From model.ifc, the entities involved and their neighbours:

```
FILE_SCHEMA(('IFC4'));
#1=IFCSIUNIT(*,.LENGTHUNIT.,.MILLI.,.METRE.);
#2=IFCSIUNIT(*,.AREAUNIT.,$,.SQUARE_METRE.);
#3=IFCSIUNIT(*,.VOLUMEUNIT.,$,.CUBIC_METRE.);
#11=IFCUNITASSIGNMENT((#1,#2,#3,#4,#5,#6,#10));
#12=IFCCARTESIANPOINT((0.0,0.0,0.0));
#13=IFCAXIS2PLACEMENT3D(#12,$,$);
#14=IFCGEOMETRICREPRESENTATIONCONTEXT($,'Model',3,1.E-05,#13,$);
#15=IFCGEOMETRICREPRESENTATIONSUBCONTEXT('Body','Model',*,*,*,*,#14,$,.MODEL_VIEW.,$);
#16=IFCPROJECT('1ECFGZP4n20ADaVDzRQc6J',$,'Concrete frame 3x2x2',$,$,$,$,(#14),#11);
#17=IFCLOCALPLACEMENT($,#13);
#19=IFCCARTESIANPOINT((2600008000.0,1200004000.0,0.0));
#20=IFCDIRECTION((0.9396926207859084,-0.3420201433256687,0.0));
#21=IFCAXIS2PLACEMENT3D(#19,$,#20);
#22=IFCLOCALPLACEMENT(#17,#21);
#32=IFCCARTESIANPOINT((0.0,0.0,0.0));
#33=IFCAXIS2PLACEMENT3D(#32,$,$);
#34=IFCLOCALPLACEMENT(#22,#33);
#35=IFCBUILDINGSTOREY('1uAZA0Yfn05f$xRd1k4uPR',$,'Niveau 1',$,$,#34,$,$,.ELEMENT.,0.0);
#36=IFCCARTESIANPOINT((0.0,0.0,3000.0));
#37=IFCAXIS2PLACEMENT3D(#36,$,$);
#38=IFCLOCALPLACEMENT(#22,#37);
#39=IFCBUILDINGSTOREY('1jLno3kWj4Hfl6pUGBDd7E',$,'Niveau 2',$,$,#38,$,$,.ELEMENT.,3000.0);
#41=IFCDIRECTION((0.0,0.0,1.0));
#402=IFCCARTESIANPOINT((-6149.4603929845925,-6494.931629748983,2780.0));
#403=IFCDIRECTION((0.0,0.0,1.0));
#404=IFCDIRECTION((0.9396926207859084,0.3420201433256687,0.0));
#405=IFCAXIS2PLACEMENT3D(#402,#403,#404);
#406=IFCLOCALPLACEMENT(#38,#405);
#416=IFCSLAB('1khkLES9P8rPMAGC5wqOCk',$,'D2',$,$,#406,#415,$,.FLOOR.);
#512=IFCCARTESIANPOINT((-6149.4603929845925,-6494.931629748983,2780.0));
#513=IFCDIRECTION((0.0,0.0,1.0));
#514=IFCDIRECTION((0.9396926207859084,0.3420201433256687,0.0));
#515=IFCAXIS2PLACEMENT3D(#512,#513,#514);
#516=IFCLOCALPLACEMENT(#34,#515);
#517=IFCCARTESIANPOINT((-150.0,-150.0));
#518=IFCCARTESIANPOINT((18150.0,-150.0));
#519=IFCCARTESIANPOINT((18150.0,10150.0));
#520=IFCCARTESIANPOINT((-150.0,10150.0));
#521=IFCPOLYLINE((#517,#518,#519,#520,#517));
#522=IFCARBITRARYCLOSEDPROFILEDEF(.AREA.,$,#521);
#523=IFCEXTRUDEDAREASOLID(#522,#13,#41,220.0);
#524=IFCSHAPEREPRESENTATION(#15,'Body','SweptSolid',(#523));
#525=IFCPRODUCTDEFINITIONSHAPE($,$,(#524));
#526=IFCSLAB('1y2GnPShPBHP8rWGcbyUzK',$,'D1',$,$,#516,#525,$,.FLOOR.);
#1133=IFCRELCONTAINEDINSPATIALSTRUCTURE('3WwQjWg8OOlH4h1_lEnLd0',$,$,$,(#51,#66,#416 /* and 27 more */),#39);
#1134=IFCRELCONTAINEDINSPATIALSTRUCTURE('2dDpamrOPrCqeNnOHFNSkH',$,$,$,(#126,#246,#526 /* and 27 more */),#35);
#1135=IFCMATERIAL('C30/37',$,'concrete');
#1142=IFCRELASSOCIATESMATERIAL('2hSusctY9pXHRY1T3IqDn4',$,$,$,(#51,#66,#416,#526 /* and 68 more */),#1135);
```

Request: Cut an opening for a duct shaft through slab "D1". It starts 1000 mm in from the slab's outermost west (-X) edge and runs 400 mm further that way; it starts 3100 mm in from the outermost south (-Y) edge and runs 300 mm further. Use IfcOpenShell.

```python
import numpy as np
import ifcopenshell
import ifcopenshell.api.feature
import ifcopenshell.api.geometry
import ifcopenshell.api.root
import ifcopenshell.geom
import ifcopenshell.util.placement
import ifcopenshell.util.representation
import ifcopenshell.util.shape
import ifcopenshell.util.unit

model = ifcopenshell.open("model.ifc")
unit_scale = ifcopenshell.util.unit.calculate_unit_scale(model)
settings = ifcopenshell.geom.settings()


def volume(element):
    """Net volume in cubic metres, openings subtracted."""
    shape = ifcopenshell.geom.create_shape(settings, element)
    return ifcopenshell.util.shape.get_volume(shape.geometry)


slab = model.by_id(526)
before = volume(slab)

# Extent in the slab's own axes, in metres. The edges named are its -X and -Y sides.
slab_shape = ifcopenshell.geom.create_shape(settings, slab)
vertices = ifcopenshell.util.shape.get_vertices(slab_shape.geometry)
x_min, y_min, bottom = vertices.min(axis=0)
top = vertices[:, 2].max()

opening = ifcopenshell.api.root.create_entity(model, ifc_class="IfcOpeningElement", name="Duct shaft opening", predefined_type="OPENING")
context = ifcopenshell.util.representation.get_context(model, "Model", "Body", "MODEL_VIEW")
width, depth = 0.4, 0.3
outline = [(0.0, 0.0), (width, 0.0), (width, depth), (0.0, depth), (0.0, 0.0)]
# Overshoot both faces by 50 mm so the cut is clean.
shape = ifcopenshell.api.geometry.add_slab_representation(
    model, context=context, depth=top - bottom + 0.1, polyline=outline
)
ifcopenshell.api.geometry.assign_representation(model, product=opening, representation=shape)

matrix = ifcopenshell.util.placement.get_local_placement(slab.ObjectPlacement)
matrix[:, 3] = matrix @ np.append(np.array([x_min + 1, y_min + 3.1, bottom - 0.05]) / unit_scale, 1.0)
ifcopenshell.api.geometry.edit_object_placement(model, product=opening, matrix=matrix, is_si=False)
ifcopenshell.api.feature.add_feature(model, feature=opening, element=slab)

after = volume(slab)

print(f"slab volume {before:.3f} -> {after:.3f} m3")

model.write("model-out.ifc")
```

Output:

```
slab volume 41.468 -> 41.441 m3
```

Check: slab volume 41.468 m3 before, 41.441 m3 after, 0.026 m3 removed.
